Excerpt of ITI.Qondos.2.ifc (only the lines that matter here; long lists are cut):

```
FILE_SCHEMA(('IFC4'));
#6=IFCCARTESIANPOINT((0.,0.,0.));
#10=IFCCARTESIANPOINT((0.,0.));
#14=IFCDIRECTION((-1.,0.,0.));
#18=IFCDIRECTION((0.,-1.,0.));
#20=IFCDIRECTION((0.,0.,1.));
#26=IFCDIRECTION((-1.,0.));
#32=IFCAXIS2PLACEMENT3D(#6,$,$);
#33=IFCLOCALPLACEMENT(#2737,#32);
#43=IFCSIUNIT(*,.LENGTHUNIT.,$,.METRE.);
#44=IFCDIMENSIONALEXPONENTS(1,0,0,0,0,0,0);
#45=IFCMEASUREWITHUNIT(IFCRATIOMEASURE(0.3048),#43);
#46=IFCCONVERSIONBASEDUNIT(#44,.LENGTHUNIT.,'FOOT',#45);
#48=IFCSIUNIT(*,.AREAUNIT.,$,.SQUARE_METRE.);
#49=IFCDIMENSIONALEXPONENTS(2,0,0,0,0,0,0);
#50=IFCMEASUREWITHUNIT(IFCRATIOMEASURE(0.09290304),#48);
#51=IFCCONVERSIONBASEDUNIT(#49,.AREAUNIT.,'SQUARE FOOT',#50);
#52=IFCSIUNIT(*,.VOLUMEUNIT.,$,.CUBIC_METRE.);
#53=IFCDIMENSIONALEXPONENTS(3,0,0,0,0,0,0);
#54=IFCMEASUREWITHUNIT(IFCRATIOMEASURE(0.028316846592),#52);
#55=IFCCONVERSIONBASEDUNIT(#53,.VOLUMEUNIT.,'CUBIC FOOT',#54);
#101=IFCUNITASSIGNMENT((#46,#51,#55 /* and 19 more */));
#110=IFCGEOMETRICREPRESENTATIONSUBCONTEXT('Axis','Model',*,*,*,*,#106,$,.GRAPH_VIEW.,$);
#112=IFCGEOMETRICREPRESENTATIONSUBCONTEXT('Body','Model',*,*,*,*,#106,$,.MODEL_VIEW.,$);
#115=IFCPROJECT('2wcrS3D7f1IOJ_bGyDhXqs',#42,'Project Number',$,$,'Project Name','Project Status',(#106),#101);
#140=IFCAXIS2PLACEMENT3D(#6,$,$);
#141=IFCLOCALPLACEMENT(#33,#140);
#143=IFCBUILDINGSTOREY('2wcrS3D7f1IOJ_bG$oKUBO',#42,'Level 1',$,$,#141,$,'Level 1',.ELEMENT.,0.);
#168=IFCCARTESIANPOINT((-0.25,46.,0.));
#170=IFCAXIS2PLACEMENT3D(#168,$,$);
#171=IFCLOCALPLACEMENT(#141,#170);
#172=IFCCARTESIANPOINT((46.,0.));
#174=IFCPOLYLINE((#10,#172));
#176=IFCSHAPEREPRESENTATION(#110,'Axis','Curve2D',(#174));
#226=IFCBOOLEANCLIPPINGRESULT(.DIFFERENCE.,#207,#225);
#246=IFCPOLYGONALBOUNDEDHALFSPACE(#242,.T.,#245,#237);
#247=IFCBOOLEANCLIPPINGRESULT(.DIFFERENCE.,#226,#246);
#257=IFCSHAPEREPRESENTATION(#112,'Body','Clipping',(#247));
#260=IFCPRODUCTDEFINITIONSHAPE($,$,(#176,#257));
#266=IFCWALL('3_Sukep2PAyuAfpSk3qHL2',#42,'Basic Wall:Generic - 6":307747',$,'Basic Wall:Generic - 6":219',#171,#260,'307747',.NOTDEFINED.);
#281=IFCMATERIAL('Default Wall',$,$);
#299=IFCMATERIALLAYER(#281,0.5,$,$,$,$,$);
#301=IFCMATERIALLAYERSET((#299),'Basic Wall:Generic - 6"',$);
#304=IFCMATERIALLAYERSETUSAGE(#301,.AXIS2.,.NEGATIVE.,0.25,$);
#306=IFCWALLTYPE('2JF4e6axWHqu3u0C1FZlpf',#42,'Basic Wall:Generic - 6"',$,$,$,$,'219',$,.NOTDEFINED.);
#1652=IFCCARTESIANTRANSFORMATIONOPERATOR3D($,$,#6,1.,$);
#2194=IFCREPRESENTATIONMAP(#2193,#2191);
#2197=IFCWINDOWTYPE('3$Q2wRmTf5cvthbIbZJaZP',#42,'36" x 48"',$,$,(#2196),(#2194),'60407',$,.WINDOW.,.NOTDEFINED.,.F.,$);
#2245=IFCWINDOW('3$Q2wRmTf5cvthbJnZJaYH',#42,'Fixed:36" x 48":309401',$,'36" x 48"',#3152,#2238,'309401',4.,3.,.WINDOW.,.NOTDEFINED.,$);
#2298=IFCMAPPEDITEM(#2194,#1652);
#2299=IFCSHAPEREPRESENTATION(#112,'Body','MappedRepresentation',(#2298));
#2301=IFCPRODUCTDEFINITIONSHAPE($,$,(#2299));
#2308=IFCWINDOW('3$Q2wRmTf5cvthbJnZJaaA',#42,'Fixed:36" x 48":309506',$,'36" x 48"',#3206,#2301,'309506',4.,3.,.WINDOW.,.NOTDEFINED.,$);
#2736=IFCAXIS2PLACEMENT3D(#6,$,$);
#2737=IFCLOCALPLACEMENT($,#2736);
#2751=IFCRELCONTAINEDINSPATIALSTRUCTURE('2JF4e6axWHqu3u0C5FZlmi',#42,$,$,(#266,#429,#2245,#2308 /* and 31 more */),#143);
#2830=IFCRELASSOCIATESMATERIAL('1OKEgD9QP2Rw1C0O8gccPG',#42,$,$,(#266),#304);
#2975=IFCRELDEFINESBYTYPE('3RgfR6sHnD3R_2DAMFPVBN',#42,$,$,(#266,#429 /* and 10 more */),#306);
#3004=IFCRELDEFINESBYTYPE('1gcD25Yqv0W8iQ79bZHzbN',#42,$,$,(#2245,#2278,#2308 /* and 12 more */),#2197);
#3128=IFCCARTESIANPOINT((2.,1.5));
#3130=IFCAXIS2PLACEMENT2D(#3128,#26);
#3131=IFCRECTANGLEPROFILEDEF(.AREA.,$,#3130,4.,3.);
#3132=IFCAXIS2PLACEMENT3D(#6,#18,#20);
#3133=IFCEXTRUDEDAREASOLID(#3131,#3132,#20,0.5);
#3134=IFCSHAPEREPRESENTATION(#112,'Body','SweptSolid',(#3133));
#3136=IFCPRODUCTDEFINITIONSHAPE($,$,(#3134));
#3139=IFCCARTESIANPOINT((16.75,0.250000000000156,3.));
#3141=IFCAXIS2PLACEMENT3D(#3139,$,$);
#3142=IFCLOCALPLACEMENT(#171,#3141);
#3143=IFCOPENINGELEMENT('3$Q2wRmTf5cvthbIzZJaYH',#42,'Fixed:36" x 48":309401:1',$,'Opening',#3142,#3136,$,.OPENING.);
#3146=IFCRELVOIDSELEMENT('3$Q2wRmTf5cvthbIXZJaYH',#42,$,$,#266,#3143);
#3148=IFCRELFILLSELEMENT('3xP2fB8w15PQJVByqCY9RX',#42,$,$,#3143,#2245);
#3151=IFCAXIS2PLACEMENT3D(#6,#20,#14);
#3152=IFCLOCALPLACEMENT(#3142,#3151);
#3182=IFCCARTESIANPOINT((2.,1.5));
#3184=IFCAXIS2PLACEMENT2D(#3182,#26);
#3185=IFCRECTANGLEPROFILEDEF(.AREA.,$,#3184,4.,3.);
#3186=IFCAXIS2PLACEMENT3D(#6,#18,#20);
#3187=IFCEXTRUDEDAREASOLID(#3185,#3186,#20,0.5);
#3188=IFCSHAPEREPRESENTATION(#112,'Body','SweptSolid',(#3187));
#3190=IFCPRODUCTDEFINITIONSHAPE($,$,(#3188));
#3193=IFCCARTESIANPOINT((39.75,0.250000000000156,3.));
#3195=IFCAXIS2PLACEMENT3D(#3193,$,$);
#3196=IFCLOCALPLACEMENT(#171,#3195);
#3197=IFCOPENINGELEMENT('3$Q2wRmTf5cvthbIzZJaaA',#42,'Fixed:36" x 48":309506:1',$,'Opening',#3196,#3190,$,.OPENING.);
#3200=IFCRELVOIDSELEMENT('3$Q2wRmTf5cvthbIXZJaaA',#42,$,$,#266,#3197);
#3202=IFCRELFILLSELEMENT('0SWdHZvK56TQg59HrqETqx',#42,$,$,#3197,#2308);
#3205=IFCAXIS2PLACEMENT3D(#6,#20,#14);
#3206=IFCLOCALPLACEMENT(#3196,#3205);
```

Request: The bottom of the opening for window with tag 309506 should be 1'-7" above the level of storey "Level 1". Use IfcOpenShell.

```python
import numpy as np
import ifcopenshell
import ifcopenshell.api.geometry
import ifcopenshell.geom
import ifcopenshell.util.element
import ifcopenshell.util.placement
import ifcopenshell.util.shape
import ifcopenshell.util.unit

model = ifcopenshell.open("ITI.Qondos.2.ifc")
unit_scale = ifcopenshell.util.unit.calculate_unit_scale(model)

window = model.by_guid("3$Q2wRmTf5cvthbJnZJaaA")
opening = window.FillsVoids[0].RelatingOpeningElement
storey = ifcopenshell.util.element.get_container(window, ifc_class="IfcBuildingStorey")
level = ifcopenshell.util.placement.get_local_placement(storey.ObjectPlacement)[2, 3]

# The opening's origin need not be at the sill, so measure its lowest point.
shape = ifcopenshell.geom.create_shape(ifcopenshell.geom.settings(), opening)
bottom = ifcopenshell.util.shape.get_shape_bottom_elevation(shape, shape.geometry) / unit_scale
dz = level + 19 * 0.0254 / unit_scale - bottom

shift = np.array([0.0, 0.0, dz])
# The window is placed relative to its opening, so it follows when the opening moves.
matrix = ifcopenshell.util.placement.get_local_placement(opening.ObjectPlacement)
matrix[:3, 3] += shift
ifcopenshell.api.geometry.edit_object_placement(
    model, product=opening, matrix=matrix, is_si=False, should_transform_children=True
)

print(f"moved by {dz * unit_scale:+.3f} m")

model.write("ITI.Qondos.2_rev.ifc")
```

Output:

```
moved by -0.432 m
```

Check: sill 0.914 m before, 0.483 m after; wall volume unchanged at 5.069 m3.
